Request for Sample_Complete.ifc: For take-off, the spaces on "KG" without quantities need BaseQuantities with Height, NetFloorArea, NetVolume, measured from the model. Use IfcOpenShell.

First a look at what the model holds.

```python
import ifcopenshell
import ifcopenshell.util.element
import ifcopenshell.util.unit

model = ifcopenshell.open("Sample_Complete.ifc")
print(model.schema)
for unit_type in ("LENGTHUNIT", "AREAUNIT", "VOLUMEUNIT"):
    print(unit_type, ifcopenshell.util.unit.calculate_unit_scale(model, unit_type))
storey = next(s for s in model.by_type("IfcBuildingStorey") if s.Name == "KG")
spaces = [e for e in ifcopenshell.util.element.get_decomposition(storey) if e.is_a("IfcSpace")]
for e in sorted(spaces, key=lambda e: e.id()):
    print(e.id(), e.is_a(), e.Name, list(ifcopenshell.util.element.get_psets(e, qtos_only=True)), sep=" | ")
```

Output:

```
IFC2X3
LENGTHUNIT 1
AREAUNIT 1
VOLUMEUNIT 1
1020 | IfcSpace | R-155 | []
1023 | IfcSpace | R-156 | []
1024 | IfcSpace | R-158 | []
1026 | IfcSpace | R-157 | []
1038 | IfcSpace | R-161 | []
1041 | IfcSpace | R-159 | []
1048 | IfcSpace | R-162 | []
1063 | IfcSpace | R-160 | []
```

```python
import ifcopenshell
import ifcopenshell.api.pset
import ifcopenshell.geom
import ifcopenshell.util.element
import ifcopenshell.util.shape
import ifcopenshell.util.unit

model = ifcopenshell.open("Sample_Complete.ifc")
unit_scale = ifcopenshell.util.unit.calculate_unit_scale(model)
area_scale = ifcopenshell.util.unit.calculate_unit_scale(model, "AREAUNIT")
volume_scale = ifcopenshell.util.unit.calculate_unit_scale(model, "VOLUMEUNIT")
settings = ifcopenshell.geom.settings()

storey = next(s for s in model.by_type("IfcBuildingStorey") if s.Name == "KG")
spaces = [e for e in ifcopenshell.util.element.get_decomposition(storey) if e.is_a("IfcSpace")]

for e in sorted(spaces, key=lambda e: e.id()):
    if ifcopenshell.util.element.get_psets(e, qtos_only=True, should_inherit=False):
        continue
    # Geometry comes back in metres, in the element's own axes.
    shape = ifcopenshell.geom.create_shape(settings, e)
    values = {
        "Height": ifcopenshell.util.shape.get_z(shape.geometry) / unit_scale,
        "NetFloorArea": ifcopenshell.util.shape.get_footprint_area(shape.geometry) / area_scale,
        "NetVolume": ifcopenshell.util.shape.get_volume(shape.geometry) / volume_scale,
    }
    qto = ifcopenshell.api.pset.add_qto(model, product=e, name="BaseQuantities")
    ifcopenshell.api.pset.edit_qto(model, qto=qto, properties=values)
    print(e.id(), {k: round(v, 3) for k, v in values.items()})

model.write("Sample_Complete_updated.ifc")
```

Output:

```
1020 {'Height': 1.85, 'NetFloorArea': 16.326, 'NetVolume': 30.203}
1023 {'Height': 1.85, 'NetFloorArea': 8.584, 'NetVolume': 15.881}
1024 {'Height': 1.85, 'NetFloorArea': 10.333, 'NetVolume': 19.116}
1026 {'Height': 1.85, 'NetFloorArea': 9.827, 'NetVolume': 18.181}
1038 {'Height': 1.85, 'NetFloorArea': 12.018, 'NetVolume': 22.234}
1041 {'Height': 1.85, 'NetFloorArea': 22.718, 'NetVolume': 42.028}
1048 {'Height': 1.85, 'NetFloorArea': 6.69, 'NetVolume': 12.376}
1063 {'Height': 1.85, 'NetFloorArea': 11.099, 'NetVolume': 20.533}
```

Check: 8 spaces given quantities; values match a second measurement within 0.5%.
